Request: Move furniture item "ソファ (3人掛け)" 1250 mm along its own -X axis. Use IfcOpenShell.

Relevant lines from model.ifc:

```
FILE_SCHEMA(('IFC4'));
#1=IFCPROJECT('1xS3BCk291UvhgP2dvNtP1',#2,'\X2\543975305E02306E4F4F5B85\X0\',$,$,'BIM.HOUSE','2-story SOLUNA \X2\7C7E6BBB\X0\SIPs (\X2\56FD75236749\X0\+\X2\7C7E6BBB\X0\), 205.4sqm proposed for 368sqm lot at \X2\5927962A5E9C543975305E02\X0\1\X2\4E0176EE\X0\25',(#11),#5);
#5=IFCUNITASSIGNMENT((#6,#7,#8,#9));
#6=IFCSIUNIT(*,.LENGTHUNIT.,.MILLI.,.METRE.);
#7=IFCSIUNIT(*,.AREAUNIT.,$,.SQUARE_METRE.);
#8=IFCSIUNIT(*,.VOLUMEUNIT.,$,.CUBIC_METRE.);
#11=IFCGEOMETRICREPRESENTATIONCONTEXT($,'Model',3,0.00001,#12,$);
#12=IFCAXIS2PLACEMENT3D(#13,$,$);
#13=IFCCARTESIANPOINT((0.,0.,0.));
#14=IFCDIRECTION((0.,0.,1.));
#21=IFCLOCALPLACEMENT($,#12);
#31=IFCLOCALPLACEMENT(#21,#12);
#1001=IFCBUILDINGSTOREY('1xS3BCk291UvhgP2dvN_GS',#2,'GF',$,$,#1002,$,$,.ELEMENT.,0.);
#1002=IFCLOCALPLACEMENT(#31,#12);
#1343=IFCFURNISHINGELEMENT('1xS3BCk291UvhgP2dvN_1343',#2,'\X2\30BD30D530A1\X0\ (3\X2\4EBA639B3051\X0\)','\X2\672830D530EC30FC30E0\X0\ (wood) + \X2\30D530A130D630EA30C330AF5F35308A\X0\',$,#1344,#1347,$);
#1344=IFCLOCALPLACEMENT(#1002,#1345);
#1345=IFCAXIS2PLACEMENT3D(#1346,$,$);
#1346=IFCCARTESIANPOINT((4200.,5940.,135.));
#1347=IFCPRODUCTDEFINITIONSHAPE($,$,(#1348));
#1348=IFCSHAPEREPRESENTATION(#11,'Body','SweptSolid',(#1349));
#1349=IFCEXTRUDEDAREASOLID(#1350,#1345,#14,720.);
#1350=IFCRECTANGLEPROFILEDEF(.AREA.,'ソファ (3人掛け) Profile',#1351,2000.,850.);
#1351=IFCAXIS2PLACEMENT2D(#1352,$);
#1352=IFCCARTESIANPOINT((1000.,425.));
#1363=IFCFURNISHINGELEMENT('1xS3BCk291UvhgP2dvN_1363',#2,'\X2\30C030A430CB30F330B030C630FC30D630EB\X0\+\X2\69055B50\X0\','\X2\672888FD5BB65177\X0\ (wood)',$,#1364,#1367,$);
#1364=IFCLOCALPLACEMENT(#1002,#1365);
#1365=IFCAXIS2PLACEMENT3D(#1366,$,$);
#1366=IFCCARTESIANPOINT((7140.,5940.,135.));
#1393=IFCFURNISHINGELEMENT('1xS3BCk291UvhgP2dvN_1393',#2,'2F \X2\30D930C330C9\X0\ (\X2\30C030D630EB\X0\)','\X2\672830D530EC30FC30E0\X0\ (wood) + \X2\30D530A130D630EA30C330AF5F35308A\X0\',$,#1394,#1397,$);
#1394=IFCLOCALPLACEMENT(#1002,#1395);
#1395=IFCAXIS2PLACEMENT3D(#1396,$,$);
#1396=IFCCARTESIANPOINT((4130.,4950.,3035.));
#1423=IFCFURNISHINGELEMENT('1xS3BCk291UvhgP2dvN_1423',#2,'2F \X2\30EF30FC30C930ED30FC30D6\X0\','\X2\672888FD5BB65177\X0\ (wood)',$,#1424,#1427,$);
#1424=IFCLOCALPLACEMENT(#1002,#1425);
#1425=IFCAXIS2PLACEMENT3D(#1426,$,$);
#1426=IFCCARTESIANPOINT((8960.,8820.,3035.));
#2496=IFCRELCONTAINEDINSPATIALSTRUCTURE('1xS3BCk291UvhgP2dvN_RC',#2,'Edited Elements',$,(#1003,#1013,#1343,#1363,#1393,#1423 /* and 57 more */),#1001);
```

```python
import ifcopenshell
import ifcopenshell.api.geometry
import ifcopenshell.util.placement
import ifcopenshell.util.unit

model = ifcopenshell.open("model.ifc")
unit_scale = ifcopenshell.util.unit.calculate_unit_scale(model)

item = model.by_id(1343)
matrix = ifcopenshell.util.placement.get_local_placement(item.ObjectPlacement)
matrix[:3, 3] -= matrix[:3, 0] * 1.25 / unit_scale
ifcopenshell.api.geometry.edit_object_placement(model, product=item, matrix=matrix, is_si=False)

print(ifcopenshell.util.placement.get_local_placement(item.ObjectPlacement).round(3) + 0.0)

model.write("model_v2.ifc")
```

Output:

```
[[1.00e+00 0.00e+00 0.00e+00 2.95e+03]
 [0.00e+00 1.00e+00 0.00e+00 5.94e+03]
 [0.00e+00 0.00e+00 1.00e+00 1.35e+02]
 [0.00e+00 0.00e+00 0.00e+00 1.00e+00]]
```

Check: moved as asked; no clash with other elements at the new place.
